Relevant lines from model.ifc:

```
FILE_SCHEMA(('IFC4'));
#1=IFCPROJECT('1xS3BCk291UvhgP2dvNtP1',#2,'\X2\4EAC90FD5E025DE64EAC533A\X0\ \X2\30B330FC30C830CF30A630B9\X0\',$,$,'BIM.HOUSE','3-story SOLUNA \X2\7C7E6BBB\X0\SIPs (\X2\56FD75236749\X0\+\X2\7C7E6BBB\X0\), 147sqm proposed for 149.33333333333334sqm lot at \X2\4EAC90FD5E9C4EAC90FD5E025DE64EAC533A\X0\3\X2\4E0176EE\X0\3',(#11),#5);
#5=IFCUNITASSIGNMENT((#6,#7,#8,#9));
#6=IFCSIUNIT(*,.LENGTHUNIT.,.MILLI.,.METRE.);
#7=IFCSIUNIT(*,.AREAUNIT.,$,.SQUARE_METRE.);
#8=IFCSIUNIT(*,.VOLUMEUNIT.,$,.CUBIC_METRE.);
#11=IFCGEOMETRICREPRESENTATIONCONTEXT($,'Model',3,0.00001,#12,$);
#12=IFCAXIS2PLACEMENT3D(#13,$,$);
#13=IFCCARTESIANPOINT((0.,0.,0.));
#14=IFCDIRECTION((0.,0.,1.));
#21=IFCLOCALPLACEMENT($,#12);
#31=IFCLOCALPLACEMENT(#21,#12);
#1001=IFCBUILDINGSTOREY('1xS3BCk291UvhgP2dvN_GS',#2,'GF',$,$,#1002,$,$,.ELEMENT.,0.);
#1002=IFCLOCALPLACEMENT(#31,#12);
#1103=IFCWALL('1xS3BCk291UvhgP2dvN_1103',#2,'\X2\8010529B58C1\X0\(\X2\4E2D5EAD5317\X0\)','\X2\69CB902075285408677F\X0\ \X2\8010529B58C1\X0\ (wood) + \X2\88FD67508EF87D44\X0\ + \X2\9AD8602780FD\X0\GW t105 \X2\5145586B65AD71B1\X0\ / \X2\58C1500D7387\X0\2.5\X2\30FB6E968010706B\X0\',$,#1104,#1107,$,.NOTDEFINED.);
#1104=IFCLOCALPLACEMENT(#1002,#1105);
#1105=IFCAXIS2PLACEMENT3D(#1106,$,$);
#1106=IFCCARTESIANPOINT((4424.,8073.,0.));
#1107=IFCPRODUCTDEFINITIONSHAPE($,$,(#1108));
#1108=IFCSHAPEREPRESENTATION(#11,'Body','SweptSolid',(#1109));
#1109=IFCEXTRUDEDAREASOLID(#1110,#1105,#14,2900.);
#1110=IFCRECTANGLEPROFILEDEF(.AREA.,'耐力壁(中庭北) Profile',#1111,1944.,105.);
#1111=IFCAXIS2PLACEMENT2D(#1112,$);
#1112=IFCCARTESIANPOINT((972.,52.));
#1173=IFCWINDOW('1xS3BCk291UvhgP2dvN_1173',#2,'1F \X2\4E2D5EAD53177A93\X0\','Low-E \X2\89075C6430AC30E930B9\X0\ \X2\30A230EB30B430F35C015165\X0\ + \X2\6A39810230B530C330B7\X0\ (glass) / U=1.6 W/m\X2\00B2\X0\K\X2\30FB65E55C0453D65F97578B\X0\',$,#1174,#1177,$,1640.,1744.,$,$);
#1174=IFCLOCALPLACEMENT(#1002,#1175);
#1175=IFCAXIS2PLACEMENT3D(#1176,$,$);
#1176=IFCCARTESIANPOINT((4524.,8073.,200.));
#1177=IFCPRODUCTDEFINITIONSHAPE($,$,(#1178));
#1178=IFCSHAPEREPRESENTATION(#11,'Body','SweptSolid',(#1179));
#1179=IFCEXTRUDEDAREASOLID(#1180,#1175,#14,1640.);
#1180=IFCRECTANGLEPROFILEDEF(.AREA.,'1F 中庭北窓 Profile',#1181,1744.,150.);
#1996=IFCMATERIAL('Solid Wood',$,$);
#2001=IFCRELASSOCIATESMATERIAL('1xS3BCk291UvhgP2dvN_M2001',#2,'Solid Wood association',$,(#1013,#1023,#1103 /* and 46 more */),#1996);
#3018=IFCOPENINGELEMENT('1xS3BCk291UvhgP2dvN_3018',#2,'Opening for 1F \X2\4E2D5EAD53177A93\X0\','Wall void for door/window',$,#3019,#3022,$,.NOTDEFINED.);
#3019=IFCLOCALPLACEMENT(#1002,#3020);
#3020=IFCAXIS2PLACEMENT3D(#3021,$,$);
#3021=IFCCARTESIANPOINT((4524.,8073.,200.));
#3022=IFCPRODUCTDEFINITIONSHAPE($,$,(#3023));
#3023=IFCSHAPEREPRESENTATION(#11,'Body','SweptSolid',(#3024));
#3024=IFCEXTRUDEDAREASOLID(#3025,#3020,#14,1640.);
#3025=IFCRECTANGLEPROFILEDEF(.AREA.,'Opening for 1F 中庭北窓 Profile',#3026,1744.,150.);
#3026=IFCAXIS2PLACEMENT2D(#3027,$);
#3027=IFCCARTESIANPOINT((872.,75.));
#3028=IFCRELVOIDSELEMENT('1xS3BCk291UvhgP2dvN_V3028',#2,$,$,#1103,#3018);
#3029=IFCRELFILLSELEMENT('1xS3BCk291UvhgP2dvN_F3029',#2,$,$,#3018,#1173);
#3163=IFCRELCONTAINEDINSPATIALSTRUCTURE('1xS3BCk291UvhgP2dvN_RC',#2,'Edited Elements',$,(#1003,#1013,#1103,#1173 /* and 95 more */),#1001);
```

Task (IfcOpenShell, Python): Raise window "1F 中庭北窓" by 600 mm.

```python
import numpy as np
import ifcopenshell
import ifcopenshell.api.geometry
import ifcopenshell.util.placement
import ifcopenshell.util.unit

model = ifcopenshell.open("model.ifc")
unit_scale = ifcopenshell.util.unit.calculate_unit_scale(model)

window = model.by_id(1173)
opening = window.FillsVoids[0].RelatingOpeningElement
dz = 600.0

shift = np.array([0.0, 0.0, dz])
# The window is not placed relative to its opening, so move both.
for product in (opening, window):
    matrix = ifcopenshell.util.placement.get_local_placement(product.ObjectPlacement)
    matrix[:3, 3] += shift
    ifcopenshell.api.geometry.edit_object_placement(model, product=product, matrix=matrix, is_si=False)

print(f"moved by {dz * unit_scale:+.3f} m")

model.write("model-out.ifc")
```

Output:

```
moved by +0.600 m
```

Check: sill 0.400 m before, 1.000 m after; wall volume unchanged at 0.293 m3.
